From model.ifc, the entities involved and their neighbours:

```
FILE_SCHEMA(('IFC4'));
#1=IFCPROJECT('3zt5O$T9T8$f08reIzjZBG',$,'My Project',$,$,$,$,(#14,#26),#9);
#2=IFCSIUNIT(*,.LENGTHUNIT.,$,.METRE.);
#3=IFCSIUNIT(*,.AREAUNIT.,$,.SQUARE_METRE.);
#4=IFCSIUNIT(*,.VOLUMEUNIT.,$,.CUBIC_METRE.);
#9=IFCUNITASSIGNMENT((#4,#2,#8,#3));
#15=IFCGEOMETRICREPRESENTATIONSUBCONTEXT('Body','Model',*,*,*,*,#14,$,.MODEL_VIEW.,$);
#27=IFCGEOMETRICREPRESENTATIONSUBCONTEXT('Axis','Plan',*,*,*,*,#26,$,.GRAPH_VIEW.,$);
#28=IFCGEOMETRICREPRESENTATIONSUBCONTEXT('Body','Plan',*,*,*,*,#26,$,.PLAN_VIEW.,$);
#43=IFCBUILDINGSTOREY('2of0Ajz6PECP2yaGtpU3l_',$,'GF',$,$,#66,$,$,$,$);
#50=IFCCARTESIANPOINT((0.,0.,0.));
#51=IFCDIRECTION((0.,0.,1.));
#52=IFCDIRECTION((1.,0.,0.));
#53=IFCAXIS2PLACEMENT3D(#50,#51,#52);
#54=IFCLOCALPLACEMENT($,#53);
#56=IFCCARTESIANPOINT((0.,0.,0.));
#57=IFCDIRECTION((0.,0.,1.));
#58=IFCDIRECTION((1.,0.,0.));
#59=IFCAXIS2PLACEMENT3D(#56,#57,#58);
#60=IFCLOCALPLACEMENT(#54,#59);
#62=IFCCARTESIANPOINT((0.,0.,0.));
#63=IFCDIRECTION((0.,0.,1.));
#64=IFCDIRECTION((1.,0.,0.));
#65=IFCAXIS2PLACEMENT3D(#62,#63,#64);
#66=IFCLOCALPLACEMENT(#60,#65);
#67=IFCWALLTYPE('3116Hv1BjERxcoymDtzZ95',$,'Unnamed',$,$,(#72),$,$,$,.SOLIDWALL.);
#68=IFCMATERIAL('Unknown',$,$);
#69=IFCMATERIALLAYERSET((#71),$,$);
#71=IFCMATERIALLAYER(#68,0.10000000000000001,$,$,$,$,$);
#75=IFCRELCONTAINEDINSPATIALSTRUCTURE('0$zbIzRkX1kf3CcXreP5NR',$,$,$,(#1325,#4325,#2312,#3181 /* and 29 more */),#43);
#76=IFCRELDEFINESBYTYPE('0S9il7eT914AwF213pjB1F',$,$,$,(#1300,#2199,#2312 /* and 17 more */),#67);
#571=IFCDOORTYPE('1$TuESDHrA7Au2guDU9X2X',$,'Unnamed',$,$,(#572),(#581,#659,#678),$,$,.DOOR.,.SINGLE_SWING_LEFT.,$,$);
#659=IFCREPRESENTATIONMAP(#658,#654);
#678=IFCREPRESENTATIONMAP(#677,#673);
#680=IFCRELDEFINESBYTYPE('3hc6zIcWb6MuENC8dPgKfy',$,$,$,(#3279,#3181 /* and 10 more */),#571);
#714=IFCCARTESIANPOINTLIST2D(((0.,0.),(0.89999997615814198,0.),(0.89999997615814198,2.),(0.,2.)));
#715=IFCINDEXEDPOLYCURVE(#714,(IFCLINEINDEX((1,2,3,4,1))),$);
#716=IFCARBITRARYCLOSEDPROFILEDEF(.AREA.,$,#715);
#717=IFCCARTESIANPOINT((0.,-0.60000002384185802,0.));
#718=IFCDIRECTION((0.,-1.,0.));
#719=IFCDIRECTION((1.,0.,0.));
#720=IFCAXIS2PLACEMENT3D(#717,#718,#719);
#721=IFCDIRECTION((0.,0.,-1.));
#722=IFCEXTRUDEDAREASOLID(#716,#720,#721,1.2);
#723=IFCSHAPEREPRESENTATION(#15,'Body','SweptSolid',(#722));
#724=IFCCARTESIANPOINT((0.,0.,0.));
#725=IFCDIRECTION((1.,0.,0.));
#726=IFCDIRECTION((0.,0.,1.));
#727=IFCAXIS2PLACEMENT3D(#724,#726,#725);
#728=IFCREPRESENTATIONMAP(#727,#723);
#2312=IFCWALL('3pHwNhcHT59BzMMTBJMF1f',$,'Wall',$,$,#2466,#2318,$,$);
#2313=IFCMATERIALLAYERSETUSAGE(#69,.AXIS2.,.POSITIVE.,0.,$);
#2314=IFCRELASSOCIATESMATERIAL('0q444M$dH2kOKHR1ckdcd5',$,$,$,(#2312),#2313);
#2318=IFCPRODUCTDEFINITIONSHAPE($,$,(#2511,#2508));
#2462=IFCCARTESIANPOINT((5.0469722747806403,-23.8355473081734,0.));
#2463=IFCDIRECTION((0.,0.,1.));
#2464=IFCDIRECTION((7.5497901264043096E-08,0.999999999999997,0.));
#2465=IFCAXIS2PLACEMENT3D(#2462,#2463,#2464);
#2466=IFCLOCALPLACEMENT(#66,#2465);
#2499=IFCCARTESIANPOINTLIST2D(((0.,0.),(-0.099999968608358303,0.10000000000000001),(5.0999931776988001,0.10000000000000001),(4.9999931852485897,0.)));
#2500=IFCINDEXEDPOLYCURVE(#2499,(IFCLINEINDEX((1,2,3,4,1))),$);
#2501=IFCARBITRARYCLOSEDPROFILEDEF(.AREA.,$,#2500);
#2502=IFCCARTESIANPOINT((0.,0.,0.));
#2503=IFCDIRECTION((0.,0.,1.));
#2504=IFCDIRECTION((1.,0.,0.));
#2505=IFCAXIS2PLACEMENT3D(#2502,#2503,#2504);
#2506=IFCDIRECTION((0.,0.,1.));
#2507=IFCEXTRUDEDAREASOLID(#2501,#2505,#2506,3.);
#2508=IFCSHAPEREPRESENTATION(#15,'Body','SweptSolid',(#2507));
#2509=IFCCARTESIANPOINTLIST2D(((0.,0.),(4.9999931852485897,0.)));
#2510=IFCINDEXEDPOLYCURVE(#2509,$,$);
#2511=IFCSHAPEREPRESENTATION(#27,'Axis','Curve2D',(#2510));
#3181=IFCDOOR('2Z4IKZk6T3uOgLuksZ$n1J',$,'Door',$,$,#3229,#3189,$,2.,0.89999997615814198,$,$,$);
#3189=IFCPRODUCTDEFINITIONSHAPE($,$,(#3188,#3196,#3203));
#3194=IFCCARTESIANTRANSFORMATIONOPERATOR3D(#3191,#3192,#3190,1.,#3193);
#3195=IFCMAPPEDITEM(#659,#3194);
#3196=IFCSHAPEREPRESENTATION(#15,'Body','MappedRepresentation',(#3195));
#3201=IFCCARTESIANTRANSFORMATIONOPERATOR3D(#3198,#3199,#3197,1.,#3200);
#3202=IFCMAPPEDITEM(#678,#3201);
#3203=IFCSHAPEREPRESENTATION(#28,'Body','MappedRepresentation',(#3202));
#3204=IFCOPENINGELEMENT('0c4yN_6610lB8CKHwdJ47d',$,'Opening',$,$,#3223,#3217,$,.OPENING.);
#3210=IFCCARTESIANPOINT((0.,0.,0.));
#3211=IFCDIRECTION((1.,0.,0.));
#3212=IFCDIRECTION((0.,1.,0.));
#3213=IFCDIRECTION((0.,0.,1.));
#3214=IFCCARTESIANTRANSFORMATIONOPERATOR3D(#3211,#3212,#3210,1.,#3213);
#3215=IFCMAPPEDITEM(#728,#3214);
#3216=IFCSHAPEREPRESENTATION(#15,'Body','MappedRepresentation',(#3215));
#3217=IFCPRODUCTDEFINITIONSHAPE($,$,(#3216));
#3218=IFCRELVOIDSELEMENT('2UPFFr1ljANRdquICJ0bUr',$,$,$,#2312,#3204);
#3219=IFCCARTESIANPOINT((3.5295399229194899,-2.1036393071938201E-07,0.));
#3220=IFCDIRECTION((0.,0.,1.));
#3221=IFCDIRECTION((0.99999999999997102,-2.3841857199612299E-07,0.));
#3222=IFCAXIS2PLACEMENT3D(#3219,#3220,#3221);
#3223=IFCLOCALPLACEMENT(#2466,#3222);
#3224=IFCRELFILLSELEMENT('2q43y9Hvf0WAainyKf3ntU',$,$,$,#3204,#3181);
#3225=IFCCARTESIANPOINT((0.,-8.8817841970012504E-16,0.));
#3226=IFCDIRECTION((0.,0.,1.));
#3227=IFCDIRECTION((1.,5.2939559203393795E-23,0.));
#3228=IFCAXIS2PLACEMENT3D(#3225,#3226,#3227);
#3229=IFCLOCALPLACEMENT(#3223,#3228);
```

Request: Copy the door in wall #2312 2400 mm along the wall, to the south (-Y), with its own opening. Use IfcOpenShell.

```python
import ifcopenshell
import ifcopenshell.api.feature
import ifcopenshell.api.geometry
import ifcopenshell.api.root
import ifcopenshell.geom
import ifcopenshell.util.element
import ifcopenshell.util.placement
import ifcopenshell.util.shape

model = ifcopenshell.open("model.ifc")
settings = ifcopenshell.geom.settings()


def volume(element):
    """Net volume in cubic metres, openings subtracted."""
    shape = ifcopenshell.geom.create_shape(settings, element)
    return ifcopenshell.util.shape.get_volume(shape.geometry)


door = model.by_guid("2Z4IKZk6T3uOgLuksZ$n1J")
opening = door.FillsVoids[0].RelatingOpeningElement
wall = opening.VoidsElements[0].RelatingBuildingElement
before = volume(wall)
shift = ifcopenshell.util.placement.get_local_placement(wall.ObjectPlacement)[:3, 0] * -2.4

# copy_class copies the void relationship, type, container and properties, but no geometry.
new_opening = ifcopenshell.api.root.copy_class(model, product=opening)
new_opening.Representation = ifcopenshell.util.element.copy_deep(
    model, opening.Representation, exclude=["IfcGeometricRepresentationContext", "IfcRepresentationMap"]
)
new_door = ifcopenshell.api.root.copy_class(model, product=door)
new_door.Representation = ifcopenshell.util.element.copy_deep(
    model, door.Representation, exclude=["IfcGeometricRepresentationContext", "IfcRepresentationMap"]
)
ifcopenshell.api.feature.add_filling(model, opening=new_opening, element=new_door)

for old, new in ((opening, new_opening), (door, new_door)):
    matrix = ifcopenshell.util.placement.get_local_placement(old.ObjectPlacement)
    matrix[:3, 3] += shift
    ifcopenshell.api.geometry.edit_object_placement(model, product=new, matrix=matrix, is_si=False)

after = volume(wall)

print(f"wall volume {before:.3f} -> {after:.3f} m3")

model.write("model_edited.ifc")
```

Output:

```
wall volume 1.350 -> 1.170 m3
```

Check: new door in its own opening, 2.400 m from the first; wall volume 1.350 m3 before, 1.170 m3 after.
